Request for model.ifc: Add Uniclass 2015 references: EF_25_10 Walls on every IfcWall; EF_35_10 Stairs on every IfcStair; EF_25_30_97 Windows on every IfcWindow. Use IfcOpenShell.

First a look at what the model holds.

```python
import ifcopenshell

model = ifcopenshell.open("model.ifc")
print(model.schema)
print("classifications:", [c.Name for c in model.by_type("IfcClassification")])
for ifc_class in ("IfcDoor", "IfcRoof", "IfcStair", "IfcWall", "IfcWindow"):
    print(ifc_class, len(model.by_type(ifc_class)))
```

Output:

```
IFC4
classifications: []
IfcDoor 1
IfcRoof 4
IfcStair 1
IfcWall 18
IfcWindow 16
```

```python
import ifcopenshell
import ifcopenshell.api.classification

model = ifcopenshell.open("model.ifc")

system = ifcopenshell.api.classification.add_classification(model, classification="Uniclass 2015")

codes = {
    "IfcWall": ("EF_25_10", "Walls"),
    "IfcStair": ("EF_35_10", "Stairs"),
    "IfcWindow": ("EF_25_30_97", "Windows"),
}
for ifc_class, (code, name) in codes.items():
    products = model.by_type(ifc_class)
    ifcopenshell.api.classification.add_reference(
        model, products=products, classification=system, identification=code, name=name
    )
    print(code, len(products))

model.write("model-out.ifc")
```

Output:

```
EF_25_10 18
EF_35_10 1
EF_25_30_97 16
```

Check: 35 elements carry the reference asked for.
